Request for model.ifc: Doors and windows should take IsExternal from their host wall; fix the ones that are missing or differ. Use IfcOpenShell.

First a look at what the model holds.

```python
import ifcopenshell
import ifcopenshell.util.element

model = ifcopenshell.open("model.ifc")
print(model.schema)
seen = {}
for e in model.by_type("IfcDoor") + model.by_type("IfcWindow"):
    if not e.FillsVoids:
        continue
    host = e.FillsVoids[0].RelatingOpeningElement.VoidsElements[0].RelatingBuildingElement
    own = ifcopenshell.util.element.get_pset(e, f"Pset_{e.is_a()[3:].removesuffix('StandardCase')}Common", "IsExternal")
    wall = ifcopenshell.util.element.get_pset(host, "Pset_WallCommon", "IsExternal")
    seen[e.is_a(), own, wall] = seen.get((e.is_a(), own, wall), 0) + 1
for (cls, own, wall), count in sorted(seen.items(), key=str):
    print(count, cls, "IsExternal:", own, "| host wall:", wall)
```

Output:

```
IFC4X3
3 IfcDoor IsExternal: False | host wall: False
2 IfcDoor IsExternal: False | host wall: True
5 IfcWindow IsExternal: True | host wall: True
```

```python
import ifcopenshell
import ifcopenshell.api.pset
import ifcopenshell.util.element

model = ifcopenshell.open("model.ifc")

count = 0
for ifc_class, pset_name in (("IfcDoor", "Pset_DoorCommon"), ("IfcWindow", "Pset_WindowCommon")):
    for e in model.by_type(ifc_class):
        if not e.FillsVoids:
            continue
        host = e.FillsVoids[0].RelatingOpeningElement.VoidsElements[0].RelatingBuildingElement
        external = ifcopenshell.util.element.get_pset(host, "Pset_WallCommon", "IsExternal")
        if external is None or ifcopenshell.util.element.get_pset(e, pset_name, "IsExternal") == external:
            continue
        pset = ifcopenshell.api.pset.add_pset(model, product=e, name=pset_name)
        ifcopenshell.api.pset.edit_pset(model, pset=pset, properties={"IsExternal": external})
        count += 1

print(count, "updated")

model.write("model_rev.ifc")
```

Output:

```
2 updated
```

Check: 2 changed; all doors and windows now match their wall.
